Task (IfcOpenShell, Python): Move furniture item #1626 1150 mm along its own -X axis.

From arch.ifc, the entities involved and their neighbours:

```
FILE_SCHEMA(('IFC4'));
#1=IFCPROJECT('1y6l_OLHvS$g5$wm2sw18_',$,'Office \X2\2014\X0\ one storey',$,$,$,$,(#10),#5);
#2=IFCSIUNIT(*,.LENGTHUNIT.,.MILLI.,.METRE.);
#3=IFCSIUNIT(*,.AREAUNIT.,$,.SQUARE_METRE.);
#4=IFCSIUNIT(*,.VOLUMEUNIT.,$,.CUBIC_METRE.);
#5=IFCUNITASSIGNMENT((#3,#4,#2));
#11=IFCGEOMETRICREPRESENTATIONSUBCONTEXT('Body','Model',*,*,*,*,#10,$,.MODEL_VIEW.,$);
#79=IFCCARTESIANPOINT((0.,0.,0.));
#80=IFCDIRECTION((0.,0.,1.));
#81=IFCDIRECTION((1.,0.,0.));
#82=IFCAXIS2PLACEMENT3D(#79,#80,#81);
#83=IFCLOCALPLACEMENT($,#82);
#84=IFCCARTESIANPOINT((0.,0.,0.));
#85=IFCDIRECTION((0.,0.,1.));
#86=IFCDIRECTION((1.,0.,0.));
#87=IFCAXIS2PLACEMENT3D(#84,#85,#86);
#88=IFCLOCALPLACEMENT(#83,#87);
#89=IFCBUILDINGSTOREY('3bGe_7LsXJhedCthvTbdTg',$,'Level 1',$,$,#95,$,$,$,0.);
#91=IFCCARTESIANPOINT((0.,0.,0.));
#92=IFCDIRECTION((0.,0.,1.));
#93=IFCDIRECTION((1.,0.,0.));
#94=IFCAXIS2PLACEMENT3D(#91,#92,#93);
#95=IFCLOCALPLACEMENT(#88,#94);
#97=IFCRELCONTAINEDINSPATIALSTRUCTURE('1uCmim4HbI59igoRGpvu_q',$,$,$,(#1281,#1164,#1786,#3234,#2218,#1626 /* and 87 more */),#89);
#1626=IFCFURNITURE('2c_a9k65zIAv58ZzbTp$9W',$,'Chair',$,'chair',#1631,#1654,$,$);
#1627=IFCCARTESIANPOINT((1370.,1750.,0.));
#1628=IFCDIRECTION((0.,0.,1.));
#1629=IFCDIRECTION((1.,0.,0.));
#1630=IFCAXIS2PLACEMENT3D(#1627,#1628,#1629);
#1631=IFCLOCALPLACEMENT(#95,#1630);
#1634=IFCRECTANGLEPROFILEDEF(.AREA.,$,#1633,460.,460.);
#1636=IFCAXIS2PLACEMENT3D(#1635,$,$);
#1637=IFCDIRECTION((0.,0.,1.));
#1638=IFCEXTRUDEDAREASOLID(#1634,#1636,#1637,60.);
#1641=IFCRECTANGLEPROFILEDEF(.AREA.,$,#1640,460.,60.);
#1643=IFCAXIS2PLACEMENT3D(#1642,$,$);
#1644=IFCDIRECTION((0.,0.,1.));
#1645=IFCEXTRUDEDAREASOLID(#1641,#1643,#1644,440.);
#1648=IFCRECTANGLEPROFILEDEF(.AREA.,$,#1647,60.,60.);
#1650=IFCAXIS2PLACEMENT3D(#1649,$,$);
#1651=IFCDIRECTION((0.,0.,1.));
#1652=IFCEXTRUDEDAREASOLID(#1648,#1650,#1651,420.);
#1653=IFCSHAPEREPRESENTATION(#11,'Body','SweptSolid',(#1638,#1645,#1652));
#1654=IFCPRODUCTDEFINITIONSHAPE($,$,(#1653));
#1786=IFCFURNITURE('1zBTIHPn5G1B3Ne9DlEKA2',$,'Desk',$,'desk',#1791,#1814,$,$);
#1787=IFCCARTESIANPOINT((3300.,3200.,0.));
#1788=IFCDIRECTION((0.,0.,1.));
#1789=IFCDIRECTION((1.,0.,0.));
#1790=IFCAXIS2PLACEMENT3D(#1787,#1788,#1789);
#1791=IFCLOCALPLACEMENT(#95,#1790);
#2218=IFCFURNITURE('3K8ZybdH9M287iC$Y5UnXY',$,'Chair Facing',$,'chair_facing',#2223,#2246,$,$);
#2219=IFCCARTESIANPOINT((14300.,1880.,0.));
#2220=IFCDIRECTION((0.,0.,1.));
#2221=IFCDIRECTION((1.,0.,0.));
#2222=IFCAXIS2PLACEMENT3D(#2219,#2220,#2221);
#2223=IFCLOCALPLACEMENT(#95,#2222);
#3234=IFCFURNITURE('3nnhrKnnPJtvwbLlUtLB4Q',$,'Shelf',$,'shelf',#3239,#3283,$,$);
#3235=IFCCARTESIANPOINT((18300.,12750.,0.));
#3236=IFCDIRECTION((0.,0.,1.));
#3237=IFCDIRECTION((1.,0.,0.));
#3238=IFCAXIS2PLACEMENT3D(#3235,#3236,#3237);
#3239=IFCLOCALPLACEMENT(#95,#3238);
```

```python
import ifcopenshell
import ifcopenshell.api.geometry
import ifcopenshell.util.placement

model = ifcopenshell.open("arch.ifc")

item = model.by_id(1626)
matrix = ifcopenshell.util.placement.get_local_placement(item.ObjectPlacement)
matrix[:3, 3] -= matrix[:3, 0] * 1150.0
ifcopenshell.api.geometry.edit_object_placement(model, product=item, matrix=matrix, is_si=False)

print(ifcopenshell.util.placement.get_local_placement(item.ObjectPlacement).round(3) + 0.0)

model.write("arch_edited.ifc")
```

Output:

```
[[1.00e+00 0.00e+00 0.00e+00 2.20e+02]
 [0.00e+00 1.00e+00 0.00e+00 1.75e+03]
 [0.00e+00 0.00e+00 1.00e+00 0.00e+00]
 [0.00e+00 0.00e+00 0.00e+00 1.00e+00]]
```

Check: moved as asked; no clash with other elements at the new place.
